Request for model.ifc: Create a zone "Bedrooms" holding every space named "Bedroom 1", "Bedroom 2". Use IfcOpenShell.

First a look at what the model holds.

```python
import ifcopenshell

model = ifcopenshell.open("model.ifc")
print(model.schema)
seen = {}
for space in model.by_type("IfcSpace"):
    seen[space.LongName] = seen.get(space.LongName, 0) + 1
for name, count in sorted(seen.items(), key=str):
    print(count, "x", name)
print("zones:", [z.Name for z in model.by_type("IfcZone")][:20])
```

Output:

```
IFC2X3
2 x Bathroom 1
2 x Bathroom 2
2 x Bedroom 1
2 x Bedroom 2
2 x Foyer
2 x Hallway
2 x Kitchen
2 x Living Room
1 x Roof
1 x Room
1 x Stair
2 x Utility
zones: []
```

```python
import ifcopenshell
import ifcopenshell.api.group
import ifcopenshell.api.root

model = ifcopenshell.open("model.ifc")

names = {"Bedroom 1", "Bedroom 2"}
spaces = [s for s in model.by_type("IfcSpace") if s.LongName in names]

zone = ifcopenshell.api.root.create_entity(model, ifc_class="IfcZone", name="Bedrooms")
ifcopenshell.api.group.assign_group(model, products=spaces, group=zone)
print(len(spaces), "spaces in", zone.Name)

model.write("model-out.ifc")
```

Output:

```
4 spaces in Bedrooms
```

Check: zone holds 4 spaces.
